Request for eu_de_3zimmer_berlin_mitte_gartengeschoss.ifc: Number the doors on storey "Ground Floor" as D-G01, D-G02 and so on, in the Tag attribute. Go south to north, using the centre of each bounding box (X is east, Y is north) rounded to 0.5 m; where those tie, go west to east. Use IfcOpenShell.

First a look at what the model holds.

```python
import ifcopenshell
import ifcopenshell.util.element
import ifcopenshell.util.placement

model = ifcopenshell.open("eu_de_3zimmer_berlin_mitte_gartengeschoss.ifc")
print(model.schema)
storey = next(s for s in model.by_type("IfcBuildingStorey") if s.Name == "Ground Floor")
doors = [e for e in ifcopenshell.util.element.get_decomposition(storey) if e.is_a("IfcDoor")]
for e in sorted(doors, key=lambda e: e.id()):
    origin = ifcopenshell.util.placement.get_local_placement(e.ObjectPlacement)[:3, 3]
    print(e.id(), e.Tag, e.Name, origin.round(2) + 0.0, sep=" | ")
```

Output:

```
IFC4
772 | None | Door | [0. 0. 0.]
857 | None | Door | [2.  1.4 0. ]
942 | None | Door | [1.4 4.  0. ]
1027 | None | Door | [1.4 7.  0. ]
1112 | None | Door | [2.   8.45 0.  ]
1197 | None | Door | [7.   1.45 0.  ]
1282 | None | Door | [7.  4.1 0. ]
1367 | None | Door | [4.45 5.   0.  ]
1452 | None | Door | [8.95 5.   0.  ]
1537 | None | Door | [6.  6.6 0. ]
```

```python
import ifcopenshell
import ifcopenshell.geom
import ifcopenshell.util.element
import ifcopenshell.util.shape

model = ifcopenshell.open("eu_de_3zimmer_berlin_mitte_gartengeschoss.ifc")
settings = ifcopenshell.geom.settings()
settings.set("use-world-coords", True)


def centre(element):
    shape = ifcopenshell.geom.create_shape(settings, element)
    return ifcopenshell.util.shape.get_bbox_centroid(shape.geometry)


storey = next(s for s in model.by_type("IfcBuildingStorey") if s.Name == "Ground Floor")
doors = [e for e in ifcopenshell.util.element.get_decomposition(storey) if e.is_a("IfcDoor")]

# Insertion points can sit at a corner or the storey origin, so sort by the geometry (in metres).
centres = {e: centre(e) for e in doors}
doors.sort(key=lambda e: (round(centres[e][1] / 0.5), centres[e][0]))

for i, e in enumerate(doors, start=1):
    number = f"D-G{i:02d}"
    e.Tag = number
    print(e.id(), number)

model.write("eu_de_3zimmer_berlin_mitte_gartengeschoss_edited.ifc")
```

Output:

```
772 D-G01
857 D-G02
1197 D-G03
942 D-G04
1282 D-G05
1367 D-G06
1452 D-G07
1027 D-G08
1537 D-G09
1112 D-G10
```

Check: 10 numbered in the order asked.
